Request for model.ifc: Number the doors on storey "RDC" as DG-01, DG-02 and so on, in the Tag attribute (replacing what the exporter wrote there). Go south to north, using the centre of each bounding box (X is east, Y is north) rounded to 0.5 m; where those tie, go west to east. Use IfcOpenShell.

First a look at what the model holds.

```python
import ifcopenshell
import ifcopenshell.util.element
import ifcopenshell.util.placement

model = ifcopenshell.open("model.ifc")
print(model.schema)
storey = next(s for s in model.by_type("IfcBuildingStorey") if s.Name == "RDC")
doors = [e for e in ifcopenshell.util.element.get_decomposition(storey) if e.is_a("IfcDoor")]
for e in sorted(doors, key=lambda e: e.id()):
    origin = ifcopenshell.util.placement.get_local_placement(e.ObjectPlacement)[:3, 3]
    print(e.id(), e.Tag, e.Name, origin.round(2) + 0.0, sep=" | ")
```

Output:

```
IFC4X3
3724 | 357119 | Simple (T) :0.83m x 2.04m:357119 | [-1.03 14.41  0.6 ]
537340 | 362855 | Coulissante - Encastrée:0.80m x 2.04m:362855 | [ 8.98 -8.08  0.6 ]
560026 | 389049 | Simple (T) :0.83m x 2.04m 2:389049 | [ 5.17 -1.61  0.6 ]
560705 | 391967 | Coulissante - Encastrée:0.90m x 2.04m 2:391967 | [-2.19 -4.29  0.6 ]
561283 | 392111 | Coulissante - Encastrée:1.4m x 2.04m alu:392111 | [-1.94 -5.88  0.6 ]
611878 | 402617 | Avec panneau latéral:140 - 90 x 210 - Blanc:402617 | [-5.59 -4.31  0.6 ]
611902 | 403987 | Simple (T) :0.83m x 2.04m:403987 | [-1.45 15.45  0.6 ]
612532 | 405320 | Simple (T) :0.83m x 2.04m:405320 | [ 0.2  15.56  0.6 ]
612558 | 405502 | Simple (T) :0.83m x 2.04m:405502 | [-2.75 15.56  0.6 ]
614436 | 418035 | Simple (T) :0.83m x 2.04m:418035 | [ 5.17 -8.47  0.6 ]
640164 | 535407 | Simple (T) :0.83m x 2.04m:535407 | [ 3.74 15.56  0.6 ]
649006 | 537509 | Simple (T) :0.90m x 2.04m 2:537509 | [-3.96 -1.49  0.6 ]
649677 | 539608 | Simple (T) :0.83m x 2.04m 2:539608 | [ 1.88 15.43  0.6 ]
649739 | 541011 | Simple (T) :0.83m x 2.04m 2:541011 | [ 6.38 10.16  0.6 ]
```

```python
import ifcopenshell
import ifcopenshell.geom
import ifcopenshell.util.element
import ifcopenshell.util.shape

model = ifcopenshell.open("model.ifc")
settings = ifcopenshell.geom.settings()
settings.set("use-world-coords", True)


def centre(element):
    shape = ifcopenshell.geom.create_shape(settings, element)
    return ifcopenshell.util.shape.get_bbox_centroid(shape.geometry)


storey = next(s for s in model.by_type("IfcBuildingStorey") if s.Name == "RDC")
doors = [e for e in ifcopenshell.util.element.get_decomposition(storey) if e.is_a("IfcDoor")]

# Insertion points can sit at a corner or the storey origin, so sort by the geometry (in metres).
centres = {e: centre(e) for e in doors}
doors.sort(key=lambda e: (round(centres[e][1] / 0.5), centres[e][0]))

for i, e in enumerate(doors, start=1):
    number = f"DG-{i:02d}"
    e.Tag = number
    print(e.id(), number)

model.write("model_updated.ifc")
```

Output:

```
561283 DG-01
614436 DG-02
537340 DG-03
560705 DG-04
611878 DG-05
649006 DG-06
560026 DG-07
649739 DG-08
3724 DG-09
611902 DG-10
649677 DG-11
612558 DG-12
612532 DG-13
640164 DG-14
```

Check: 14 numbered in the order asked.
